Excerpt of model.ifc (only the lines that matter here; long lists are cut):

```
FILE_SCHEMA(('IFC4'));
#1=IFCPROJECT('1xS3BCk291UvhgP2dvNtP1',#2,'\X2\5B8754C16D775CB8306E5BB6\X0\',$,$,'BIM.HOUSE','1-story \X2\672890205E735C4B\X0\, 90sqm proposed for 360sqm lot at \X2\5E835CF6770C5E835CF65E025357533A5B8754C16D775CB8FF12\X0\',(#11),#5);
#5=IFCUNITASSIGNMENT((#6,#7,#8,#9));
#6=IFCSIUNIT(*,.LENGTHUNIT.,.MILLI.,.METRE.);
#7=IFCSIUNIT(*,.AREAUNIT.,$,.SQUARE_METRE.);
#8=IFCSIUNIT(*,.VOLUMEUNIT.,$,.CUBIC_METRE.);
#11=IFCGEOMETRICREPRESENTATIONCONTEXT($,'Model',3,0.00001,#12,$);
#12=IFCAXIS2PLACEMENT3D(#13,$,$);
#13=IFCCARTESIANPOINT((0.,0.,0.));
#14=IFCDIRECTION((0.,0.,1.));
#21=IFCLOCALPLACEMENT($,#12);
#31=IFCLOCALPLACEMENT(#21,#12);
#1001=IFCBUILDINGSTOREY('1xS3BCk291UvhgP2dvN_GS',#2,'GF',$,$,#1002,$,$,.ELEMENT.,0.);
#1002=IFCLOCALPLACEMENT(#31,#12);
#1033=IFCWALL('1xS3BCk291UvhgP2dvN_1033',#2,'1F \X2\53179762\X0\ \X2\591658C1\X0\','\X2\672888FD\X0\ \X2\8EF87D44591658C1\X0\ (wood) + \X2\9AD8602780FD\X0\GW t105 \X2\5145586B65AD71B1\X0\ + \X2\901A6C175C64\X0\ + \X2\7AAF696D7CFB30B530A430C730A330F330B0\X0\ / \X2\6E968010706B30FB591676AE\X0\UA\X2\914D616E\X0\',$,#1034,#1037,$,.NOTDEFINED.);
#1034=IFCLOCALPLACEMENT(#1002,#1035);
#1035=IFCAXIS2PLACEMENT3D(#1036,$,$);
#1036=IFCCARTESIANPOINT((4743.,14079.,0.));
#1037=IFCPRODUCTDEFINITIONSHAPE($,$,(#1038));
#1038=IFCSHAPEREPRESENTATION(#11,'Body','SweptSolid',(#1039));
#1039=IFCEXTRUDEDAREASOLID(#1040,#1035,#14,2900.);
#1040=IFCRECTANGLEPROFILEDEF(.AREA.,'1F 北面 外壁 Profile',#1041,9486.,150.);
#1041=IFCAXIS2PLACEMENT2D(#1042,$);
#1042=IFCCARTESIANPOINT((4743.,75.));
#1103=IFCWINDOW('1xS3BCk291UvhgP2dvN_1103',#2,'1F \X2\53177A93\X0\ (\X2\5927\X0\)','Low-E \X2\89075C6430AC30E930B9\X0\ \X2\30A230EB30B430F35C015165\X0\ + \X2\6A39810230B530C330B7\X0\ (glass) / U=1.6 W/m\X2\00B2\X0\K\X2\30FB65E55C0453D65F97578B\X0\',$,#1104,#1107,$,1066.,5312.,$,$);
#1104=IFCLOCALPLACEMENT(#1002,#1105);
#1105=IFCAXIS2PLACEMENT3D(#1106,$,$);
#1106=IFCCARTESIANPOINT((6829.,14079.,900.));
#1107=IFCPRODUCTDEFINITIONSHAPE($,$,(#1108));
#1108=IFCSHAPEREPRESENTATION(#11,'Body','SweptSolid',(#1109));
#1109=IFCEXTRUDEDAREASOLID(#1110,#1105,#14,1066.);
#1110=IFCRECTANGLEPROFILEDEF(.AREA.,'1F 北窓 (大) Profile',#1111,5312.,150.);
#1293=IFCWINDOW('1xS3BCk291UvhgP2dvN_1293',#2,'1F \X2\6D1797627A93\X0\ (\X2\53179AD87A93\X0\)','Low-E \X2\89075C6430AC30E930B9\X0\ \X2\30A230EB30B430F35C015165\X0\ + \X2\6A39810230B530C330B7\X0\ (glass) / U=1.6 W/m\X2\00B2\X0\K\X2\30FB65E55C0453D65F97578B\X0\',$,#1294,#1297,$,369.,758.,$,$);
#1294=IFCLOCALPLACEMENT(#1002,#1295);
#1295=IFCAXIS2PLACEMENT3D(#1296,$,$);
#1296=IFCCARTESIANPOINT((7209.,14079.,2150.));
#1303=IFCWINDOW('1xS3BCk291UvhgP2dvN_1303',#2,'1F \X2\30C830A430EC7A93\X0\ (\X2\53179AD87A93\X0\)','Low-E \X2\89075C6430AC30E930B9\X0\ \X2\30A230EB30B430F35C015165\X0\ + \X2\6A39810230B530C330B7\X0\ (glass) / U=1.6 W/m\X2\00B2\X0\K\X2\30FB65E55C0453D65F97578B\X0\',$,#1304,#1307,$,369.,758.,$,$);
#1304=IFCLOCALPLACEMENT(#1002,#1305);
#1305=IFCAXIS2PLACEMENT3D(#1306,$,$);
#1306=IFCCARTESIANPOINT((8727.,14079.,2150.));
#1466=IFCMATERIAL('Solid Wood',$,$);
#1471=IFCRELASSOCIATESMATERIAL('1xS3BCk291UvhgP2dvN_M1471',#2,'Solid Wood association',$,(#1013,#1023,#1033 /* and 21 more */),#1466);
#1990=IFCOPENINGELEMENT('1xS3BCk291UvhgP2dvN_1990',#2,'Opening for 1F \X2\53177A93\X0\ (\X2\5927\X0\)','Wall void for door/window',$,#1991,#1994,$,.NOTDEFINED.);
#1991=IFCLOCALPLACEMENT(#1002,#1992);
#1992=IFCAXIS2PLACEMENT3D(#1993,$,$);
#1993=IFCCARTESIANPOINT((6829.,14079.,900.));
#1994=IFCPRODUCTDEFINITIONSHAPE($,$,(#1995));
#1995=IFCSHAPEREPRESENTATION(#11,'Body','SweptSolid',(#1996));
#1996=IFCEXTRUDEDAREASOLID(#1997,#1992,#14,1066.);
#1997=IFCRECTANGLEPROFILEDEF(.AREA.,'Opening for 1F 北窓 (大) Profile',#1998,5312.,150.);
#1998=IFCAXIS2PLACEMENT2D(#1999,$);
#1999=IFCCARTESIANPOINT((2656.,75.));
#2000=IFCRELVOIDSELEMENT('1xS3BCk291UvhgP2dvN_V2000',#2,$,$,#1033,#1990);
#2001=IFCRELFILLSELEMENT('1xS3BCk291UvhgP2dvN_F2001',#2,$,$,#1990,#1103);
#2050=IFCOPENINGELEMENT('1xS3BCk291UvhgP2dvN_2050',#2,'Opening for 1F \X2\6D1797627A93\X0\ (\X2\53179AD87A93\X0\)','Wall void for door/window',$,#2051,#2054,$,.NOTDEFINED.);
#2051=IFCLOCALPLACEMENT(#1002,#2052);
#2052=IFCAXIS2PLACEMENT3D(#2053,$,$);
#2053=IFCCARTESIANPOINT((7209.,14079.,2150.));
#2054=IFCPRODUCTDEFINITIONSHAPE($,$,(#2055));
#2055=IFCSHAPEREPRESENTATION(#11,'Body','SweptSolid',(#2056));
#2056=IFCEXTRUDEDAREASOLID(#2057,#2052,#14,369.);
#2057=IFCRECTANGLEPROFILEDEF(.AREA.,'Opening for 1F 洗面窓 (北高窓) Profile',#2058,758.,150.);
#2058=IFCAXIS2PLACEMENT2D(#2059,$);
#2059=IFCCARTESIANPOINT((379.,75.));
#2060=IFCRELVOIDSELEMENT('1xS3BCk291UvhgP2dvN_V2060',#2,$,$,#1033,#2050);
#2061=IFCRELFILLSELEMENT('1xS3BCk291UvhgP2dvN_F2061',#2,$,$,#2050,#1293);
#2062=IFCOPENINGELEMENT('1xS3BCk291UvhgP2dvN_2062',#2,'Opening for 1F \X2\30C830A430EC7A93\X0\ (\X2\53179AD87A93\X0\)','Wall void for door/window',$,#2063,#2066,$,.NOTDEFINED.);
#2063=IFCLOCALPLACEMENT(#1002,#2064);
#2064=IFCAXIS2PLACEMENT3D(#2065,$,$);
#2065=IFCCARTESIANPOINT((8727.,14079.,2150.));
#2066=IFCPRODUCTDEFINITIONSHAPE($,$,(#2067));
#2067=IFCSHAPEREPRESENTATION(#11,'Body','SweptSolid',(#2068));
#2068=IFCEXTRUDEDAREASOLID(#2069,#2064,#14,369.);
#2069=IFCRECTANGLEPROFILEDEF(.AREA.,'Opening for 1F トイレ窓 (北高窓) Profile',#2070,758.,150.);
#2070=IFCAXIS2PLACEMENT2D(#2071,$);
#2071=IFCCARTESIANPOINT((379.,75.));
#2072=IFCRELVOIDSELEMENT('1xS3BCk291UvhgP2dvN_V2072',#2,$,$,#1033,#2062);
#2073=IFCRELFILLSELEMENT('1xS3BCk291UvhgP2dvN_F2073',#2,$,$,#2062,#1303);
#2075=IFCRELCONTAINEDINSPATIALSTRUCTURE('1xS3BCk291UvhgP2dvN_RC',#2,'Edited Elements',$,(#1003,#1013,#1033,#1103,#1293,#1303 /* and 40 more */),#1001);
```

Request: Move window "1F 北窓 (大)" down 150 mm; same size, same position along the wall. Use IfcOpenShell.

```python
import numpy as np
import ifcopenshell
import ifcopenshell.api.geometry
import ifcopenshell.util.placement
import ifcopenshell.util.unit

model = ifcopenshell.open("model.ifc")
unit_scale = ifcopenshell.util.unit.calculate_unit_scale(model)

window = model.by_guid("1xS3BCk291UvhgP2dvN_1103")
opening = window.FillsVoids[0].RelatingOpeningElement
dz = -150.0

shift = np.array([0.0, 0.0, dz])
# The window is not placed relative to its opening, so move both.
for product in (opening, window):
    matrix = ifcopenshell.util.placement.get_local_placement(product.ObjectPlacement)
    matrix[:3, 3] += shift
    ifcopenshell.api.geometry.edit_object_placement(model, product=product, matrix=matrix, is_si=False)

print(f"moved by {dz * unit_scale:+.3f} m")

model.write("model_rev.ifc")
```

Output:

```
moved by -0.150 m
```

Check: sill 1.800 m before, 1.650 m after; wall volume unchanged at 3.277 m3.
